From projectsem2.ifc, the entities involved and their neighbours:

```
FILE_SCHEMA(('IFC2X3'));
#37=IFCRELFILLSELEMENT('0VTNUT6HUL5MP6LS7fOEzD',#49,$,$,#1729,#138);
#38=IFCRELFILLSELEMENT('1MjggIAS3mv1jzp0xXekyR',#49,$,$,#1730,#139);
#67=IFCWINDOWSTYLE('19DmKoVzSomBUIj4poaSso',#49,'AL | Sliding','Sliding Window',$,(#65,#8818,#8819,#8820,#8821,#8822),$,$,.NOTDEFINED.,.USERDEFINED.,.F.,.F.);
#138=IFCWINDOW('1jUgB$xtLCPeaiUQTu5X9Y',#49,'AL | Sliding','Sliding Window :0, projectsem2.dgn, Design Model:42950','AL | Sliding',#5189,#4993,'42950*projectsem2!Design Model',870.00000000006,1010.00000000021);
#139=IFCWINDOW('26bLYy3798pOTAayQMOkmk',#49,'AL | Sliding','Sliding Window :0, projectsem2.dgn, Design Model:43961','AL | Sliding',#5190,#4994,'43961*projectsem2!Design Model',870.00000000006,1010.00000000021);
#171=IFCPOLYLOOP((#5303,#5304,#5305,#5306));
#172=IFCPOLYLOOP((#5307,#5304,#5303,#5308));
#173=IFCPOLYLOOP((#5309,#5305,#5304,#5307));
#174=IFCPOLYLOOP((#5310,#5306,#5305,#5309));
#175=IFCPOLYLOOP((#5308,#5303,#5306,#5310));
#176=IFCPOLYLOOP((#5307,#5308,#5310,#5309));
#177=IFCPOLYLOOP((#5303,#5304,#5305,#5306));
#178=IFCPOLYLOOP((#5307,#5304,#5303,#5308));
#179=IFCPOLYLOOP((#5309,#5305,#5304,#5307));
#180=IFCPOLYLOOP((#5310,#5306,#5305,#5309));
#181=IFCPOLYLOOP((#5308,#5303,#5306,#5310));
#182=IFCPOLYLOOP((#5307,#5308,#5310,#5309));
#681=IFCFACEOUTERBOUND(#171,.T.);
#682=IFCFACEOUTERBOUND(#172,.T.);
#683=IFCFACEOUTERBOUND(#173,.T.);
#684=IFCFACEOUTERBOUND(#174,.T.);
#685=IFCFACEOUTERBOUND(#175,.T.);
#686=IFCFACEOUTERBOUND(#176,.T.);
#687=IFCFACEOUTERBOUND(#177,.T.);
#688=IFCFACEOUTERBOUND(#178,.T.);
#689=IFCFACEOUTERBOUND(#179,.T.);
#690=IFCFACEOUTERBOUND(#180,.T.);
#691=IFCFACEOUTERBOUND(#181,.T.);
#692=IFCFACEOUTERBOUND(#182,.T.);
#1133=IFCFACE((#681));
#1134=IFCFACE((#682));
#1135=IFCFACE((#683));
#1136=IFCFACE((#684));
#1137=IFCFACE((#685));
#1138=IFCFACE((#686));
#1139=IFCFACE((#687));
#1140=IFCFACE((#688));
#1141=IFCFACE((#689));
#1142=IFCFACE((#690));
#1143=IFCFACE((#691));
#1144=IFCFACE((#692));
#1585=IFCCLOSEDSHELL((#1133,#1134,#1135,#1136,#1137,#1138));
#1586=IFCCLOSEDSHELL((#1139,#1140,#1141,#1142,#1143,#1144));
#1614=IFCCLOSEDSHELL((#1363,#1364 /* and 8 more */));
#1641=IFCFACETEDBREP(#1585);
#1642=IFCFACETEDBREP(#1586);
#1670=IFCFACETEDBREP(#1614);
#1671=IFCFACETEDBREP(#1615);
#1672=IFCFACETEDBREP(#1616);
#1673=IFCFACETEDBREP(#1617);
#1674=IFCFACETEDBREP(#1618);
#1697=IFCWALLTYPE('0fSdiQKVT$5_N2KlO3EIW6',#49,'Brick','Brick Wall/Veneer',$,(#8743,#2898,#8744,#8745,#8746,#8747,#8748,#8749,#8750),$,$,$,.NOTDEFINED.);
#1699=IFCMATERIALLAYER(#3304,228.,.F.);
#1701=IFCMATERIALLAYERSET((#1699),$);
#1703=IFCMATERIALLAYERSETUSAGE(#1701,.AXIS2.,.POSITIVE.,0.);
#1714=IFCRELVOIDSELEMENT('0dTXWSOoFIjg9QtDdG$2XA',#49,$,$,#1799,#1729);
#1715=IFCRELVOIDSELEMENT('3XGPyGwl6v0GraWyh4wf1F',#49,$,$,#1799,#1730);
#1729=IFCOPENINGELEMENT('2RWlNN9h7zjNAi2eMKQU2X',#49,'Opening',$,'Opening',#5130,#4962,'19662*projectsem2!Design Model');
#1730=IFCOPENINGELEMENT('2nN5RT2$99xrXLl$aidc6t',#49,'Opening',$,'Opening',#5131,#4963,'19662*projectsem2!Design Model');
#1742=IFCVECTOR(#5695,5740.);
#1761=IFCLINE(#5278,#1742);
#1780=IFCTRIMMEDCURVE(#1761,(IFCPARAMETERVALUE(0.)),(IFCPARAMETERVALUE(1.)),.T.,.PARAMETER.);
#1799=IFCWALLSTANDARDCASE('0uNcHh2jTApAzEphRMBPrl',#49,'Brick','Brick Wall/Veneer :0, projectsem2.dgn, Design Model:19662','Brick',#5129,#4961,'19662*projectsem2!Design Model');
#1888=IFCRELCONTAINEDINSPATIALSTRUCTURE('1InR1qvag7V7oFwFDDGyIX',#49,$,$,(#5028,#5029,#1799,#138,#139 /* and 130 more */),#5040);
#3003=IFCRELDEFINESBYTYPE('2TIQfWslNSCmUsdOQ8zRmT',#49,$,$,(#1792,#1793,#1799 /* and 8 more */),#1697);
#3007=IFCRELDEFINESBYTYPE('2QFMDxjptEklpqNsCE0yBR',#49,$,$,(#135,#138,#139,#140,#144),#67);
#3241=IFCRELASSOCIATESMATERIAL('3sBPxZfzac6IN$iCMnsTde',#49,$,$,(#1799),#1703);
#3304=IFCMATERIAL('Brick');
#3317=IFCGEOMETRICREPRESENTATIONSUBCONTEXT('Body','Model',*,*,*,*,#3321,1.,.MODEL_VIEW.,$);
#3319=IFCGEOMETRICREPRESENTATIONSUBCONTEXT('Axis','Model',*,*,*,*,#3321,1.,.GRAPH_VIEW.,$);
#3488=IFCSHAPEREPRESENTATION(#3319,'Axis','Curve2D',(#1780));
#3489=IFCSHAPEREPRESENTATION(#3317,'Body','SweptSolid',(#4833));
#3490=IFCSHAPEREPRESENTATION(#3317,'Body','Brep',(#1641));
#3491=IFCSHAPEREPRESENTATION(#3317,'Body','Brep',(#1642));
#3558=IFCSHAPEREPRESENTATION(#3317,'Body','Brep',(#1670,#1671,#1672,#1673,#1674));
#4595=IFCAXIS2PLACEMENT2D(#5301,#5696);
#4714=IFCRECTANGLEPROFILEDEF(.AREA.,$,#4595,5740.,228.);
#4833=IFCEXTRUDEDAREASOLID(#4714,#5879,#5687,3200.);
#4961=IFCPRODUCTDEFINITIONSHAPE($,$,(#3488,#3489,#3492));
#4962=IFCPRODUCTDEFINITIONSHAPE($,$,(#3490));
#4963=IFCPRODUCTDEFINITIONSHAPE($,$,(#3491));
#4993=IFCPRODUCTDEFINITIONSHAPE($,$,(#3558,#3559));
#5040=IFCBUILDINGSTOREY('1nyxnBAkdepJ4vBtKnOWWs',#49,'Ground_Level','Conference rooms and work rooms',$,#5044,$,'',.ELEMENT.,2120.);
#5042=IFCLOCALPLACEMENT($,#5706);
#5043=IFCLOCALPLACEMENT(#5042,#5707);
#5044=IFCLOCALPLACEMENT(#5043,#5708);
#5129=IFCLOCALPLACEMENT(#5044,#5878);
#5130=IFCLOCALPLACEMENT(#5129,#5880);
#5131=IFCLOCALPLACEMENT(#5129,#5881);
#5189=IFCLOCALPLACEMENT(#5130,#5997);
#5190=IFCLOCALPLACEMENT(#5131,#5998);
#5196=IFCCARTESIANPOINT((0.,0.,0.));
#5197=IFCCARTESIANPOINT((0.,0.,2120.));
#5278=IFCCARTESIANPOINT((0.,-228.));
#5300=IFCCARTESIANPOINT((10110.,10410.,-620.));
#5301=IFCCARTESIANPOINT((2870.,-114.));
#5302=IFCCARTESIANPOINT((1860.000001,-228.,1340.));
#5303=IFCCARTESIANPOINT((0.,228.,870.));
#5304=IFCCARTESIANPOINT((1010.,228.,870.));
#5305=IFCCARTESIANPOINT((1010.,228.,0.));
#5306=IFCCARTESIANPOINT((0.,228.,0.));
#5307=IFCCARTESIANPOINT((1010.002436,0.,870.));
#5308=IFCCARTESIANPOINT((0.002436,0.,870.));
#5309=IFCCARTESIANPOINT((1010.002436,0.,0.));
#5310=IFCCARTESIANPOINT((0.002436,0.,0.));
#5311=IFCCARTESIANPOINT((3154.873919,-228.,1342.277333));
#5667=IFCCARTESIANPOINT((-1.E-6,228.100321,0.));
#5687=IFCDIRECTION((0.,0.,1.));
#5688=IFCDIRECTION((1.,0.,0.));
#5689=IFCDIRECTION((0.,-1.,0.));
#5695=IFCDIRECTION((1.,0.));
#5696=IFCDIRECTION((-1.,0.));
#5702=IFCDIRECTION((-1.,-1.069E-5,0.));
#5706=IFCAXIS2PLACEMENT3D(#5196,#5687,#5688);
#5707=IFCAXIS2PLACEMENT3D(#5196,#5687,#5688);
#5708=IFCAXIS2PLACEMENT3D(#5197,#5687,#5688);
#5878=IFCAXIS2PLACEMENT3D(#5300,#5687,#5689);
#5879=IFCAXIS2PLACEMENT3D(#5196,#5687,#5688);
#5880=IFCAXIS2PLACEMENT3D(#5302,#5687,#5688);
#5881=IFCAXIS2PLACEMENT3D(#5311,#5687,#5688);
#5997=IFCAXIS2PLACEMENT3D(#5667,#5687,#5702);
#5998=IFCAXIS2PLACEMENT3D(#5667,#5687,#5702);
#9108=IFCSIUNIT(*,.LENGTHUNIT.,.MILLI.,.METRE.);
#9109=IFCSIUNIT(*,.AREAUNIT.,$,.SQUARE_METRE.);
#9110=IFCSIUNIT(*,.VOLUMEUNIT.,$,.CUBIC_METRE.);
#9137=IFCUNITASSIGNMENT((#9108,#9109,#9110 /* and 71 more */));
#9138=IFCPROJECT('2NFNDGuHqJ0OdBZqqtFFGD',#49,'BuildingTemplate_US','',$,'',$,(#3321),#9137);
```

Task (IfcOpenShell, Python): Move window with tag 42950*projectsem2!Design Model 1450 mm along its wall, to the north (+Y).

```python
import ifcopenshell
import ifcopenshell.api.geometry
import ifcopenshell.util.placement
import ifcopenshell.util.unit

model = ifcopenshell.open("projectsem2.ifc")
unit_scale = ifcopenshell.util.unit.calculate_unit_scale(model)

window = model.by_guid("1jUgB$xtLCPeaiUQTu5X9Y")
opening = window.FillsVoids[0].RelatingOpeningElement
wall = opening.VoidsElements[0].RelatingBuildingElement

wall_matrix = ifcopenshell.util.placement.get_local_placement(wall.ObjectPlacement)
shift = wall_matrix[:3, 0] * -1.45 / unit_scale
before = ifcopenshell.util.placement.get_local_placement(window.ObjectPlacement)[:3, 3].copy()

# The window is placed relative to its opening, so it follows when the opening moves.
matrix = ifcopenshell.util.placement.get_local_placement(opening.ObjectPlacement)
matrix[:3, 3] += shift
ifcopenshell.api.geometry.edit_object_placement(
    model, product=opening, matrix=matrix, is_si=False, should_transform_children=True
)

after = ifcopenshell.util.placement.get_local_placement(window.ObjectPlacement)[:3, 3]
print("window moved by", (after - before).round(3) + 0.0)

model.write("projectsem2-out.ifc")
```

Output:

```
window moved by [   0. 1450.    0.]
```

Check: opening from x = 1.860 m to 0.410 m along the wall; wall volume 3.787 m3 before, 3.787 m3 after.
